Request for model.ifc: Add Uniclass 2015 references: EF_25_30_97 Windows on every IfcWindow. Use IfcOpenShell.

First a look at what the model holds.

```python
import ifcopenshell

model = ifcopenshell.open("model.ifc")
print(model.schema)
print("classifications:", [c.Name for c in model.by_type("IfcClassification")])
for ifc_class in ("IfcDoor", "IfcRoof", "IfcStair", "IfcWall", "IfcWindow"):
    print(ifc_class, len(model.by_type(ifc_class)))
```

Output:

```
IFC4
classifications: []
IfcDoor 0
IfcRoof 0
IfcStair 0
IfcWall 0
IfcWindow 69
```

```python
import ifcopenshell
import ifcopenshell.api.classification

model = ifcopenshell.open("model.ifc")

system = ifcopenshell.api.classification.add_classification(model, classification="Uniclass 2015")

codes = {
    "IfcWindow": ("EF_25_30_97", "Windows"),
}
for ifc_class, (code, name) in codes.items():
    products = model.by_type(ifc_class)
    ifcopenshell.api.classification.add_reference(
        model, products=products, classification=system, identification=code, name=name
    )
    print(code, len(products))

model.write("model_edited.ifc")
```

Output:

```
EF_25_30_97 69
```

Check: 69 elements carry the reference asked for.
